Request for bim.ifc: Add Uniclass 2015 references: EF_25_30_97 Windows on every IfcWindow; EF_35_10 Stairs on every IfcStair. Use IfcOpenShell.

First a look at what the model holds.

```python
import ifcopenshell

model = ifcopenshell.open("bim.ifc")
print(model.schema)
print("classifications:", [c.Name for c in model.by_type("IfcClassification")])
for ifc_class in ("IfcDoor", "IfcRoof", "IfcStair", "IfcWall", "IfcWindow"):
    print(ifc_class, len(model.by_type(ifc_class)))
```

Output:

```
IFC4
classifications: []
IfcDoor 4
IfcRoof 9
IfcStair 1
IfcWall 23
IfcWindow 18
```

```python
import ifcopenshell
import ifcopenshell.api.classification

model = ifcopenshell.open("bim.ifc")

system = ifcopenshell.api.classification.add_classification(model, classification="Uniclass 2015")

codes = {
    "IfcWindow": ("EF_25_30_97", "Windows"),
    "IfcStair": ("EF_35_10", "Stairs"),
}
for ifc_class, (code, name) in codes.items():
    products = model.by_type(ifc_class)
    ifcopenshell.api.classification.add_reference(
        model, products=products, classification=system, identification=code, name=name
    )
    print(code, len(products))

model.write("bim_rev.ifc")
```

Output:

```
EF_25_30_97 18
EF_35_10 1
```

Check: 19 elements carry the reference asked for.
